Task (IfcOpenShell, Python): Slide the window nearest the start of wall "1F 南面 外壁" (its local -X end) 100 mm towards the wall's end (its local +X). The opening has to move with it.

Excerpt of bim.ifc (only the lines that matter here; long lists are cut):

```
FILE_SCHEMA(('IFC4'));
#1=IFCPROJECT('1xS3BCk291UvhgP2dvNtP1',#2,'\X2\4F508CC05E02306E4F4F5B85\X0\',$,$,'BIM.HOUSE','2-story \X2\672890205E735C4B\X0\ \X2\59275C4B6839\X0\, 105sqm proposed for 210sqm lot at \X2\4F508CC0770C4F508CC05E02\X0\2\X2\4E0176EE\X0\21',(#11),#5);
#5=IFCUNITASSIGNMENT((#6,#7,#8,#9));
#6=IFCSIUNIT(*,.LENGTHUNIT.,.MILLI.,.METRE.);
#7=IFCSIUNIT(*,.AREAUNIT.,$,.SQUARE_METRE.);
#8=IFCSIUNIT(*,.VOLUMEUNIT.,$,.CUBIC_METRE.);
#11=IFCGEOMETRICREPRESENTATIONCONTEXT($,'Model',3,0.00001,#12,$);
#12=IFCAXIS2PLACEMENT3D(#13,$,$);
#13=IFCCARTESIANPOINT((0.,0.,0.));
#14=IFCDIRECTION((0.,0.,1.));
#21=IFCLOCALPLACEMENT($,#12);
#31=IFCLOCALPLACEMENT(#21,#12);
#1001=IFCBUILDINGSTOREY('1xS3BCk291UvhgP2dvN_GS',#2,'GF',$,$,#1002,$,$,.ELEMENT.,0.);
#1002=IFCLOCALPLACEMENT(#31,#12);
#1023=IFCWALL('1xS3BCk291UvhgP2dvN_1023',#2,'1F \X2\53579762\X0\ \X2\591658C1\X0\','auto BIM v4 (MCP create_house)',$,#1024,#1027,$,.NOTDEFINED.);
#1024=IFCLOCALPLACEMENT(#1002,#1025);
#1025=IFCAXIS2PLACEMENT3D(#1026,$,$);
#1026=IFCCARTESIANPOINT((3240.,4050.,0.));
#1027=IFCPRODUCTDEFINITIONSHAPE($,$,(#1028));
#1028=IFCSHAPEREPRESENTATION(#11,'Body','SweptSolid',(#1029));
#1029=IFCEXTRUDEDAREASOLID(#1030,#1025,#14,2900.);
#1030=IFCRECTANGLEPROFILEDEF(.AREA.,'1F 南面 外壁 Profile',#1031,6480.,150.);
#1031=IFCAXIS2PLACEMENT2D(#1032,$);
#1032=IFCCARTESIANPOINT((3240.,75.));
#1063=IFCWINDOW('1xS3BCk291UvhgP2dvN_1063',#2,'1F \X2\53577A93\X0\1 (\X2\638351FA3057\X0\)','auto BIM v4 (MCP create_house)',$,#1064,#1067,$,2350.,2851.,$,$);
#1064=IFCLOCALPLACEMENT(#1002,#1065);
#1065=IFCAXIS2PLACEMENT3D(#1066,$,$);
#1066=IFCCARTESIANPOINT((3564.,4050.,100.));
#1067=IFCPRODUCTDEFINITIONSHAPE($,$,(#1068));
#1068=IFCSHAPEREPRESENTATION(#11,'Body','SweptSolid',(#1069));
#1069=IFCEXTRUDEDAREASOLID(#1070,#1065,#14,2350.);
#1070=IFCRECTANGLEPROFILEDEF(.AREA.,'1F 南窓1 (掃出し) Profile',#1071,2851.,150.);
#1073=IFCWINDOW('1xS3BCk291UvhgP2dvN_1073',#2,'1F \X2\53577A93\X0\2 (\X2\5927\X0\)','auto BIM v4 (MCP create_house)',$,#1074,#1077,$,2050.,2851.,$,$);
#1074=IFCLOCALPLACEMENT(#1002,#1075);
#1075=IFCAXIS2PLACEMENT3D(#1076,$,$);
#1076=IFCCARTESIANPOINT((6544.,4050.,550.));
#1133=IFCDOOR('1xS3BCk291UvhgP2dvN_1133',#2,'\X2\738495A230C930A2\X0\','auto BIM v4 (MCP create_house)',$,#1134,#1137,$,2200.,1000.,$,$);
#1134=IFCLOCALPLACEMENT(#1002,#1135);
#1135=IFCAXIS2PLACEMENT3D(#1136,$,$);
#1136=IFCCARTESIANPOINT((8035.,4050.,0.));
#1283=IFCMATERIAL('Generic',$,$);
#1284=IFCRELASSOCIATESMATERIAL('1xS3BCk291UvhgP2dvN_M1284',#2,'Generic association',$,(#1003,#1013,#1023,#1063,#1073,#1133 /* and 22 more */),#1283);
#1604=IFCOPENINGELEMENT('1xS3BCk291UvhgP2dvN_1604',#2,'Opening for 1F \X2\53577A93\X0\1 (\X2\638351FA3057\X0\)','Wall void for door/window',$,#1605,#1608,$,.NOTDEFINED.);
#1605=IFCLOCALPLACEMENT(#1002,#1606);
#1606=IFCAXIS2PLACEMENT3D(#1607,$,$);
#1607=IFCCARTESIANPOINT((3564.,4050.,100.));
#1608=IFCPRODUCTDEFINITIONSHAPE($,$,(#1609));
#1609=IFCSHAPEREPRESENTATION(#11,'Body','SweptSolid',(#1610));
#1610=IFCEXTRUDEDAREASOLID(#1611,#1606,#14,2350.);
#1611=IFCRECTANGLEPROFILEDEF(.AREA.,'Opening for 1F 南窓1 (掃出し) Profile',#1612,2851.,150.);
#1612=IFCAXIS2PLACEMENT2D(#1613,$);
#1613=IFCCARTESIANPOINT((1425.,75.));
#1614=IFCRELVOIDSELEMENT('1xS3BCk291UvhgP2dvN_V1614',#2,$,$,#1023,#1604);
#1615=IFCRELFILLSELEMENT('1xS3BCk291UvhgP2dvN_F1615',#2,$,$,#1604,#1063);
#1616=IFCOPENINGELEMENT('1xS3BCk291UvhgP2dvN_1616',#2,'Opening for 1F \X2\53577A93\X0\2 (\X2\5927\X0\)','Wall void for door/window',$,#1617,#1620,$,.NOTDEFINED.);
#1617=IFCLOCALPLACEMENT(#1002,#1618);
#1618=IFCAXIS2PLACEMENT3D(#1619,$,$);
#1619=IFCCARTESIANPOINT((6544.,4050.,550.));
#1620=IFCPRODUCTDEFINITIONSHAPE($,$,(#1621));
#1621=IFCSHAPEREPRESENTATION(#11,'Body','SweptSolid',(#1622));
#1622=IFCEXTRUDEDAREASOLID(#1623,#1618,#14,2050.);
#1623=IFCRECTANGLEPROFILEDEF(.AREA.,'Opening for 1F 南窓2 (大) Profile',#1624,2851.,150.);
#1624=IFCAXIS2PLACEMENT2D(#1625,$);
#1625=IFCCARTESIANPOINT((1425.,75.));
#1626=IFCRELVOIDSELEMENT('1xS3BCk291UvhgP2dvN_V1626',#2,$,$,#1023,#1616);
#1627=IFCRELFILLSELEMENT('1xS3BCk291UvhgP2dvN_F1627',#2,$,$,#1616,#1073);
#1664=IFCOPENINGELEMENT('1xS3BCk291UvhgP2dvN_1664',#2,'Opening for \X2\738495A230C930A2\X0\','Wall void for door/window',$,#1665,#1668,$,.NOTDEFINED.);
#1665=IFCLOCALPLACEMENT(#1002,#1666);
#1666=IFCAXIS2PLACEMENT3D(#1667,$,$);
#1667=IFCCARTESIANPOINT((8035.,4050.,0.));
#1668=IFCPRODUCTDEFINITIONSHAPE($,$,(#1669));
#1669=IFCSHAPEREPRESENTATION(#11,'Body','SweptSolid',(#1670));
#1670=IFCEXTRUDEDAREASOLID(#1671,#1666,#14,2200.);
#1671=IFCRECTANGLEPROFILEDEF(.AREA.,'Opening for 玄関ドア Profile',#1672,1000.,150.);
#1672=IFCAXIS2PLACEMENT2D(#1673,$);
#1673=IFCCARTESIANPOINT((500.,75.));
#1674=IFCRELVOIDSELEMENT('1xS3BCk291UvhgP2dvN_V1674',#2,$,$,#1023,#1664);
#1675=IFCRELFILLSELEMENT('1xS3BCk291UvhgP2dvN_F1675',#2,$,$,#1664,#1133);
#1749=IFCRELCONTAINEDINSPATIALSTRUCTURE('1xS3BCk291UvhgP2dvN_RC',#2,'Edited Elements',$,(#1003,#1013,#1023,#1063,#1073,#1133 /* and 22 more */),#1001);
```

```python
import ifcopenshell
import ifcopenshell.api.geometry
import ifcopenshell.util.placement
import ifcopenshell.util.unit

model = ifcopenshell.open("bim.ifc")
unit_scale = ifcopenshell.util.unit.calculate_unit_scale(model)

window = model.by_id(1063)
opening = window.FillsVoids[0].RelatingOpeningElement
wall = opening.VoidsElements[0].RelatingBuildingElement

wall_matrix = ifcopenshell.util.placement.get_local_placement(wall.ObjectPlacement)
shift = wall_matrix[:3, 0] * 0.1 / unit_scale
before = ifcopenshell.util.placement.get_local_placement(window.ObjectPlacement)[:3, 3].copy()

# The window is not placed relative to its opening, so move both.
for product in (opening, window):
    matrix = ifcopenshell.util.placement.get_local_placement(product.ObjectPlacement)
    matrix[:3, 3] += shift
    ifcopenshell.api.geometry.edit_object_placement(model, product=product, matrix=matrix, is_si=False)

after = ifcopenshell.util.placement.get_local_placement(window.ObjectPlacement)[:3, 3]
print("window moved by", (after - before).round(3) + 0.0)

model.write("bim_rev.ifc")
```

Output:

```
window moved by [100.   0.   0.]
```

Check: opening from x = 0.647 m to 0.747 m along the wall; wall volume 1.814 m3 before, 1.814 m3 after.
